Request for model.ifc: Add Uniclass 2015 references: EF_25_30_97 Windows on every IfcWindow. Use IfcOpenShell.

First a look at what the model holds.

```python
import ifcopenshell

model = ifcopenshell.open("model.ifc")
print(model.schema)
print("classifications:", [c.Name for c in model.by_type("IfcClassification")])
for ifc_class in ("IfcDoor", "IfcRoof", "IfcStair", "IfcWall", "IfcWindow"):
    print(ifc_class, len(model.by_type(ifc_class)))
```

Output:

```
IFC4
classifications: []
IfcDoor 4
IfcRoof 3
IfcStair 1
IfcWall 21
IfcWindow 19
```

```python
import ifcopenshell
import ifcopenshell.api.classification

model = ifcopenshell.open("model.ifc")

system = ifcopenshell.api.classification.add_classification(model, classification="Uniclass 2015")

codes = {
    "IfcWindow": ("EF_25_30_97", "Windows"),
}
for ifc_class, (code, name) in codes.items():
    products = model.by_type(ifc_class)
    ifcopenshell.api.classification.add_reference(
        model, products=products, classification=system, identification=code, name=name
    )
    print(code, len(products))

model.write("model_v2.ifc")
```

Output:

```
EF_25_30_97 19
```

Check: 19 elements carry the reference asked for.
